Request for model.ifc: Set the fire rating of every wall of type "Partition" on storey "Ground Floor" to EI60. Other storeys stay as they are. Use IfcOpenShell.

First a look at what the model holds.

```python
import ifcopenshell
import ifcopenshell.util.element

model = ifcopenshell.open("model.ifc")
print(model.schema)
storey = next(s for s in model.by_type("IfcBuildingStorey") if s.Name == "Ground Floor")
walls = [e for e in ifcopenshell.util.element.get_decomposition(storey) if e.is_a("IfcWall")]
seen = {}
for e in walls:
    element_type = ifcopenshell.util.element.get_type(e)
    key = (element_type.Name if element_type != e and element_type else None, ifcopenshell.util.element.get_pset(e, "Pset_WallCommon", "FireRating"))
    seen[key] = seen.get(key, 0) + 1
for (name, value), count in sorted(seen.items(), key=str):
    print(count, "x", name, "|", value)
```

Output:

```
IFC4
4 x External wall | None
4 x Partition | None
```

```python
import ifcopenshell
import ifcopenshell.api.pset
import ifcopenshell.util.element

model = ifcopenshell.open("model.ifc")

storey = next(s for s in model.by_type("IfcBuildingStorey") if s.Name == "Ground Floor")
walls = [e for e in ifcopenshell.util.element.get_decomposition(storey) if e.is_a("IfcWall")]

count = 0
for e in walls:
    element_type = ifcopenshell.util.element.get_type(e)
    if element_type in (None, e) or element_type.Name != "Partition":
        continue
    # add_pset returns the element's existing set when there is one.
    pset = ifcopenshell.api.pset.add_pset(model, product=e, name="Pset_WallCommon")
    ifcopenshell.api.pset.edit_pset(model, pset=pset, properties={"FireRating": "EI60"})
    count += 1

print(count, "walls updated")

model.write("model_updated.ifc")
```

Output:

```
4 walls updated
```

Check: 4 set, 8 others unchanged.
